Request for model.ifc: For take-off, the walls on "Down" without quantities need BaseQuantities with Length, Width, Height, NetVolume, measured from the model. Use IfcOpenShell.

First a look at what the model holds.

```python
import ifcopenshell
import ifcopenshell.util.element
import ifcopenshell.util.unit

model = ifcopenshell.open("model.ifc")
print(model.schema)
for unit_type in ("LENGTHUNIT", "AREAUNIT", "VOLUMEUNIT"):
    print(unit_type, ifcopenshell.util.unit.calculate_unit_scale(model, unit_type))
storey = next(s for s in model.by_type("IfcBuildingStorey") if s.Name == "Down")
walls = [e for e in ifcopenshell.util.element.get_decomposition(storey) if e.is_a("IfcWall")]
for e in sorted(walls, key=lambda e: e.id()):
    print(e.id(), e.is_a(), e.Name, list(ifcopenshell.util.element.get_psets(e, qtos_only=True)), sep=" | ")
```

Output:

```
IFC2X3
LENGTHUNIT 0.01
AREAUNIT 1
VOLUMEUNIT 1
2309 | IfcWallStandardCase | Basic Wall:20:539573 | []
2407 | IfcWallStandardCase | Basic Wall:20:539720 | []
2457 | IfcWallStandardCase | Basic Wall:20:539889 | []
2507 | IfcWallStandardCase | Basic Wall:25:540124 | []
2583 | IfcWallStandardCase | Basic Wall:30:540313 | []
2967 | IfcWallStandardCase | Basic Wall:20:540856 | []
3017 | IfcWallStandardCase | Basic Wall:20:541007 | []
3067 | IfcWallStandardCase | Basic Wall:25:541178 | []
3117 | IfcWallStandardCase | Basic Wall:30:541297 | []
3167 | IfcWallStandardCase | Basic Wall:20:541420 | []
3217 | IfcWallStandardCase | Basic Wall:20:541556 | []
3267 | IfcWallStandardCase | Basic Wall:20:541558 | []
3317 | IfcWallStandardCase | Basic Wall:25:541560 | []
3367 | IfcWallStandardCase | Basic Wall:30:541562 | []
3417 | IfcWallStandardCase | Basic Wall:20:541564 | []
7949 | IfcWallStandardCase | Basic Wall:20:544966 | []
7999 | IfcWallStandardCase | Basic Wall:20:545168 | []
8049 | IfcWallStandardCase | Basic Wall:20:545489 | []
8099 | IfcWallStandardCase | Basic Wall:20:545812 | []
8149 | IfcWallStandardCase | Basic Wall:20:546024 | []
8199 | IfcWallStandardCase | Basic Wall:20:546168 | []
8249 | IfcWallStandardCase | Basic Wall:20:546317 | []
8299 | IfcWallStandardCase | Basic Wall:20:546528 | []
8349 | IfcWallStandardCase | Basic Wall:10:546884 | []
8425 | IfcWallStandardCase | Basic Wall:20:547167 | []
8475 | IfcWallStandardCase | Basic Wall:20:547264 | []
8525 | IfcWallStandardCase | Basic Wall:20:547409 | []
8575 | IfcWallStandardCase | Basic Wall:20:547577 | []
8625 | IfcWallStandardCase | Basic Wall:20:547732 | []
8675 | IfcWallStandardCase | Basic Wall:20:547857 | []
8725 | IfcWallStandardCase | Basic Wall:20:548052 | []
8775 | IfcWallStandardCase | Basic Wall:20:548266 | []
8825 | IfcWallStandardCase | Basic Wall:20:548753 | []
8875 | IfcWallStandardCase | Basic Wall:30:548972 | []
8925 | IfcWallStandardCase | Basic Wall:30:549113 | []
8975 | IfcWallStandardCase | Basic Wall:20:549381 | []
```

```python
import ifcopenshell
import ifcopenshell.api.pset
import ifcopenshell.geom
import ifcopenshell.util.element
import ifcopenshell.util.shape
import ifcopenshell.util.unit

model = ifcopenshell.open("model.ifc")
unit_scale = ifcopenshell.util.unit.calculate_unit_scale(model)
volume_scale = ifcopenshell.util.unit.calculate_unit_scale(model, "VOLUMEUNIT")
settings = ifcopenshell.geom.settings()

storey = next(s for s in model.by_type("IfcBuildingStorey") if s.Name == "Down")
walls = [e for e in ifcopenshell.util.element.get_decomposition(storey) if e.is_a("IfcWall")]

for e in sorted(walls, key=lambda e: e.id()):
    if ifcopenshell.util.element.get_psets(e, qtos_only=True, should_inherit=False):
        continue
    # Geometry comes back in metres, in the element's own axes.
    shape = ifcopenshell.geom.create_shape(settings, e)
    values = {
        "Length": ifcopenshell.util.shape.get_x(shape.geometry) / unit_scale,
        "Width": ifcopenshell.util.shape.get_y(shape.geometry) / unit_scale,
        "Height": ifcopenshell.util.shape.get_z(shape.geometry) / unit_scale,
        "NetVolume": ifcopenshell.util.shape.get_volume(shape.geometry) / volume_scale,
    }
    qto = ifcopenshell.api.pset.add_qto(model, product=e, name="BaseQuantities")
    ifcopenshell.api.pset.edit_qto(model, qto=qto, properties=values)
    print(e.id(), {k: round(v, 3) for k, v in values.items()})

model.write("model_v2.ifc")
```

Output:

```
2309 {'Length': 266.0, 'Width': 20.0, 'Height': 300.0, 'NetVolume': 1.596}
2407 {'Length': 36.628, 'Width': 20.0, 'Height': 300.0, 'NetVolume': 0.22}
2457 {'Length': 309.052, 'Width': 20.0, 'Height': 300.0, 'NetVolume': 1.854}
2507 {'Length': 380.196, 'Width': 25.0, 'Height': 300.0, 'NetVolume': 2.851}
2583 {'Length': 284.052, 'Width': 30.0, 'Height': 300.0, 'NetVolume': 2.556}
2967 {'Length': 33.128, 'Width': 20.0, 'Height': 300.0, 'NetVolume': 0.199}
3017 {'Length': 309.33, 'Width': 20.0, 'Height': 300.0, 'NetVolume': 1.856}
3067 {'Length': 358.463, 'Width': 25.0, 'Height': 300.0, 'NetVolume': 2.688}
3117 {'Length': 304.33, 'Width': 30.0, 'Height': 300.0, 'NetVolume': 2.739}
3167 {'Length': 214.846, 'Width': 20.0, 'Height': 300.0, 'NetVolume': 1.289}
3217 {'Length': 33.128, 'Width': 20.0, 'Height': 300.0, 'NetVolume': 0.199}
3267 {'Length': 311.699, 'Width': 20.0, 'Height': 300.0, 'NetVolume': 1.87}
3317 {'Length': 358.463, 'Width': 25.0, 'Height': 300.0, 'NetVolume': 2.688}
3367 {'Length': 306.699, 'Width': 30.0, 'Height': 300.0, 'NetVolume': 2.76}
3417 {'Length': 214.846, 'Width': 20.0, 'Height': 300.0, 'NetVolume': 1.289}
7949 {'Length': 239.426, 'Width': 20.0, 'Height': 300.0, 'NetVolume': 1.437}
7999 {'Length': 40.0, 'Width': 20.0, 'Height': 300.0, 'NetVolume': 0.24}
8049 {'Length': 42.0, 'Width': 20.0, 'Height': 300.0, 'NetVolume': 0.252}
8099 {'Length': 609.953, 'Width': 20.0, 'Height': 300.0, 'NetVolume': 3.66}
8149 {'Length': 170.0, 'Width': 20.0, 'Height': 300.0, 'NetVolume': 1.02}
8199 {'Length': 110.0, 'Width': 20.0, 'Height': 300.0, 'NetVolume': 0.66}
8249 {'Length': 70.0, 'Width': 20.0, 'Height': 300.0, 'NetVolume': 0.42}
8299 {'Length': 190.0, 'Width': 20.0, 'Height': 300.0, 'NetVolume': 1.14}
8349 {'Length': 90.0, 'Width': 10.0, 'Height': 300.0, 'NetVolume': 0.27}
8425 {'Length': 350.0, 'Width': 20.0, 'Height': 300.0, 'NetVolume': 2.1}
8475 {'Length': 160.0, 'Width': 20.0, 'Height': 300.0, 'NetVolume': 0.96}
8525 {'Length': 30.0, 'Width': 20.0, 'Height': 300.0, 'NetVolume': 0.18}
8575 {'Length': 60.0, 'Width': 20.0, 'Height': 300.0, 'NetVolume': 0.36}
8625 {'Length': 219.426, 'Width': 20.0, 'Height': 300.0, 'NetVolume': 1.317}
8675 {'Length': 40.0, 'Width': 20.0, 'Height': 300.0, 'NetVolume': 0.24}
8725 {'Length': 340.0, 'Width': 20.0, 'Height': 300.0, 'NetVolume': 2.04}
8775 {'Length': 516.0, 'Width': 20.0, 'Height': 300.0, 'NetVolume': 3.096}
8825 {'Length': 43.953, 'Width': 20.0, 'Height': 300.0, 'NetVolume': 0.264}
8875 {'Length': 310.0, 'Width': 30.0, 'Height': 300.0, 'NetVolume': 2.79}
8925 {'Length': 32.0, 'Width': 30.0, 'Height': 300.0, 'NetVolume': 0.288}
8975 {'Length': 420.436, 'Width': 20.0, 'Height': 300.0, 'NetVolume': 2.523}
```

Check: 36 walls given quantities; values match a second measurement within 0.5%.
